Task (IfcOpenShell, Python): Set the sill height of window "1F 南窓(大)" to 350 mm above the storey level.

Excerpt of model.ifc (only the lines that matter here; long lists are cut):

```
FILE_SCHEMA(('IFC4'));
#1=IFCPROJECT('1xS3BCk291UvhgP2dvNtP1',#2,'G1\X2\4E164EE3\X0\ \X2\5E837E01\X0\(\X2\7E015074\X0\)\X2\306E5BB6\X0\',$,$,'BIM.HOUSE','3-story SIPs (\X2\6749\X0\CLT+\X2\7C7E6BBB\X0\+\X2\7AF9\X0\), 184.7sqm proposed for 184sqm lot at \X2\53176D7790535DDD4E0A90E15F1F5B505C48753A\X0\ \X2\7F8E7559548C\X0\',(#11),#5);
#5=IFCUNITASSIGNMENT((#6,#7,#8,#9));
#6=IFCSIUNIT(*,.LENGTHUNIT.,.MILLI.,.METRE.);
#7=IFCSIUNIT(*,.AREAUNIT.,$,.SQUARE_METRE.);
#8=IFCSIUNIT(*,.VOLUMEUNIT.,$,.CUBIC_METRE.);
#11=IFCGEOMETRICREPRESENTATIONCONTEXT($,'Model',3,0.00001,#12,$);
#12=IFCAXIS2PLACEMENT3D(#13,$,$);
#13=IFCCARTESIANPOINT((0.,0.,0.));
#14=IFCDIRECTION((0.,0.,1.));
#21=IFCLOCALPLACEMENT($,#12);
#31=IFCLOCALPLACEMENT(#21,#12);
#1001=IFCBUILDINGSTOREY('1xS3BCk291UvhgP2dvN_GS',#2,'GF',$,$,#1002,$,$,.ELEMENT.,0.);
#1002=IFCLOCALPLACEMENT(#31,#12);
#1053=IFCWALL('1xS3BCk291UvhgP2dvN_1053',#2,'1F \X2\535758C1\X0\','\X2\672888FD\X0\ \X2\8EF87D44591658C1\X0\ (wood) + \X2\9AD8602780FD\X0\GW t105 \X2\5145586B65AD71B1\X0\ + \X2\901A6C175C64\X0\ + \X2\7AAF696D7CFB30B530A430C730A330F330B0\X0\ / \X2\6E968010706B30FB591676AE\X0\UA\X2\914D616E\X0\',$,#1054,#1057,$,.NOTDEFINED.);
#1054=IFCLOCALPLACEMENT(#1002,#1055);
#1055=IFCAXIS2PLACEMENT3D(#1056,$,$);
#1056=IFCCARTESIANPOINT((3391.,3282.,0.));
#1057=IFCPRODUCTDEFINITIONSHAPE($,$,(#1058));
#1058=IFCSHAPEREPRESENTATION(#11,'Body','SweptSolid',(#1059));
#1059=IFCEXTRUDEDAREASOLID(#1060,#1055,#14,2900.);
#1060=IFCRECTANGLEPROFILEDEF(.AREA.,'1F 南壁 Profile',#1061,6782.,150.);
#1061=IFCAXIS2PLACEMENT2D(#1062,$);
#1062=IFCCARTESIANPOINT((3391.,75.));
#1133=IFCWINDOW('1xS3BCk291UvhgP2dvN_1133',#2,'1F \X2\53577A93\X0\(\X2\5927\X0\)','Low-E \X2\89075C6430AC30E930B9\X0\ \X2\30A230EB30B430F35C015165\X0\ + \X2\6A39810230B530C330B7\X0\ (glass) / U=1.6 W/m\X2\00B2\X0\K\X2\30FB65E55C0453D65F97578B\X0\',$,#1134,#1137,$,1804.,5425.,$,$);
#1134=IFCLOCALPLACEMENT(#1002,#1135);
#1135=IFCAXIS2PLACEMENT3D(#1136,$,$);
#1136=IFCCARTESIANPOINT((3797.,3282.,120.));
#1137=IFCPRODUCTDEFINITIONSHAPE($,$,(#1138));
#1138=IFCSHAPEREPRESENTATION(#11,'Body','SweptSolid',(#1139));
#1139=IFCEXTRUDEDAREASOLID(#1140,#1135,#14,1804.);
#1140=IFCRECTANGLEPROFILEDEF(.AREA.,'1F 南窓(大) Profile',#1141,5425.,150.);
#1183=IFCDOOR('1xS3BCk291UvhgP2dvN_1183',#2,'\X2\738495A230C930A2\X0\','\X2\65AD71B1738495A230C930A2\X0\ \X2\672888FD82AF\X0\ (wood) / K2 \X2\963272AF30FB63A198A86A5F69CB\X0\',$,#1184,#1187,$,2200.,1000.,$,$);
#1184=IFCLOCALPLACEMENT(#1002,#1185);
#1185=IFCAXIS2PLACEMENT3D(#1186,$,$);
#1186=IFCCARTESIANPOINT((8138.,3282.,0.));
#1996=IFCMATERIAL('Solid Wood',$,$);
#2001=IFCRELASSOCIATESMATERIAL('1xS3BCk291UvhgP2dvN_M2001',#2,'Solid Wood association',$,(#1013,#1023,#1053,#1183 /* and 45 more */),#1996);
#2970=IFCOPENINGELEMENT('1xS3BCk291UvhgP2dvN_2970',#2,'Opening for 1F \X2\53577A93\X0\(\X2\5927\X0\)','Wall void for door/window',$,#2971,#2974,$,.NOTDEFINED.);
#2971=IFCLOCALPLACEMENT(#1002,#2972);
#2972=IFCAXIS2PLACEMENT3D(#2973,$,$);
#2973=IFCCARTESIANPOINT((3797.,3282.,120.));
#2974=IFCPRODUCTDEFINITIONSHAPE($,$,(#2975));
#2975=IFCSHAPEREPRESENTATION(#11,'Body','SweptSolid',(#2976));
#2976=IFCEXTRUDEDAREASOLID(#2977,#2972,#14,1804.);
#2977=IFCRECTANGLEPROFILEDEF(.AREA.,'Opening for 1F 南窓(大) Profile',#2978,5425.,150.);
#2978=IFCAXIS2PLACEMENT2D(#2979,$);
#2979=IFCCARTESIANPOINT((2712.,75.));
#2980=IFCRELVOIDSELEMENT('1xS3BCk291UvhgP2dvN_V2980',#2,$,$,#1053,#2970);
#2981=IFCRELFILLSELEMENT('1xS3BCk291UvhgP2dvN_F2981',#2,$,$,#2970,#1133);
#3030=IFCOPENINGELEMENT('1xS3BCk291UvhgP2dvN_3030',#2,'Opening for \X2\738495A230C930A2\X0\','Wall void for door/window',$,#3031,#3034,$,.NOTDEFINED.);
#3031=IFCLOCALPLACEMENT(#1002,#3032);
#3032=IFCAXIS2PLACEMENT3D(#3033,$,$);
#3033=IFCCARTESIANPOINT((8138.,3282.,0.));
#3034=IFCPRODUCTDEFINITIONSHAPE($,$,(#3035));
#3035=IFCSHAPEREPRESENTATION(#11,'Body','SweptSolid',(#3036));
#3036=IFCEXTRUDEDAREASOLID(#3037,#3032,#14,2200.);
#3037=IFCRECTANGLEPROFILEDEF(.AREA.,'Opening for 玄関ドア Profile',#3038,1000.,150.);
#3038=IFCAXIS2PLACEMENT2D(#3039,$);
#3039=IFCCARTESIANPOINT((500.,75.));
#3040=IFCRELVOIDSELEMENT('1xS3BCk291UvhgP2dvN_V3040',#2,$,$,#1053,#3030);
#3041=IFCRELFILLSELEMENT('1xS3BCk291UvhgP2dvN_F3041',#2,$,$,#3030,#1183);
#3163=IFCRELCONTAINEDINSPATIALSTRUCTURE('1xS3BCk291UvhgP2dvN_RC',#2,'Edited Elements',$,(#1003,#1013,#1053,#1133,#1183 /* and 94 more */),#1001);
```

```python
import numpy as np
import ifcopenshell
import ifcopenshell.api.geometry
import ifcopenshell.geom
import ifcopenshell.util.element
import ifcopenshell.util.placement
import ifcopenshell.util.shape
import ifcopenshell.util.unit

model = ifcopenshell.open("model.ifc")
unit_scale = ifcopenshell.util.unit.calculate_unit_scale(model)

window = model.by_guid("1xS3BCk291UvhgP2dvN_1133")
opening = window.FillsVoids[0].RelatingOpeningElement
storey = ifcopenshell.util.element.get_container(window, ifc_class="IfcBuildingStorey")
level = ifcopenshell.util.placement.get_local_placement(storey.ObjectPlacement)[2, 3]

# The opening's origin need not be at the sill, so measure its lowest point.
shape = ifcopenshell.geom.create_shape(ifcopenshell.geom.settings(), opening)
bottom = ifcopenshell.util.shape.get_shape_bottom_elevation(shape, shape.geometry) / unit_scale
dz = level + 0.35 / unit_scale - bottom

shift = np.array([0.0, 0.0, dz])
# The window is not placed relative to its opening, so move both.
for product in (opening, window):
    matrix = ifcopenshell.util.placement.get_local_placement(product.ObjectPlacement)
    matrix[:3, 3] += shift
    ifcopenshell.api.geometry.edit_object_placement(model, product=product, matrix=matrix, is_si=False)

print(f"moved by {dz * unit_scale:+.3f} m")

model.write("model_updated.ifc")
```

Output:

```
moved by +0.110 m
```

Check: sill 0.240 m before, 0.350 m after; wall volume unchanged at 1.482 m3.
